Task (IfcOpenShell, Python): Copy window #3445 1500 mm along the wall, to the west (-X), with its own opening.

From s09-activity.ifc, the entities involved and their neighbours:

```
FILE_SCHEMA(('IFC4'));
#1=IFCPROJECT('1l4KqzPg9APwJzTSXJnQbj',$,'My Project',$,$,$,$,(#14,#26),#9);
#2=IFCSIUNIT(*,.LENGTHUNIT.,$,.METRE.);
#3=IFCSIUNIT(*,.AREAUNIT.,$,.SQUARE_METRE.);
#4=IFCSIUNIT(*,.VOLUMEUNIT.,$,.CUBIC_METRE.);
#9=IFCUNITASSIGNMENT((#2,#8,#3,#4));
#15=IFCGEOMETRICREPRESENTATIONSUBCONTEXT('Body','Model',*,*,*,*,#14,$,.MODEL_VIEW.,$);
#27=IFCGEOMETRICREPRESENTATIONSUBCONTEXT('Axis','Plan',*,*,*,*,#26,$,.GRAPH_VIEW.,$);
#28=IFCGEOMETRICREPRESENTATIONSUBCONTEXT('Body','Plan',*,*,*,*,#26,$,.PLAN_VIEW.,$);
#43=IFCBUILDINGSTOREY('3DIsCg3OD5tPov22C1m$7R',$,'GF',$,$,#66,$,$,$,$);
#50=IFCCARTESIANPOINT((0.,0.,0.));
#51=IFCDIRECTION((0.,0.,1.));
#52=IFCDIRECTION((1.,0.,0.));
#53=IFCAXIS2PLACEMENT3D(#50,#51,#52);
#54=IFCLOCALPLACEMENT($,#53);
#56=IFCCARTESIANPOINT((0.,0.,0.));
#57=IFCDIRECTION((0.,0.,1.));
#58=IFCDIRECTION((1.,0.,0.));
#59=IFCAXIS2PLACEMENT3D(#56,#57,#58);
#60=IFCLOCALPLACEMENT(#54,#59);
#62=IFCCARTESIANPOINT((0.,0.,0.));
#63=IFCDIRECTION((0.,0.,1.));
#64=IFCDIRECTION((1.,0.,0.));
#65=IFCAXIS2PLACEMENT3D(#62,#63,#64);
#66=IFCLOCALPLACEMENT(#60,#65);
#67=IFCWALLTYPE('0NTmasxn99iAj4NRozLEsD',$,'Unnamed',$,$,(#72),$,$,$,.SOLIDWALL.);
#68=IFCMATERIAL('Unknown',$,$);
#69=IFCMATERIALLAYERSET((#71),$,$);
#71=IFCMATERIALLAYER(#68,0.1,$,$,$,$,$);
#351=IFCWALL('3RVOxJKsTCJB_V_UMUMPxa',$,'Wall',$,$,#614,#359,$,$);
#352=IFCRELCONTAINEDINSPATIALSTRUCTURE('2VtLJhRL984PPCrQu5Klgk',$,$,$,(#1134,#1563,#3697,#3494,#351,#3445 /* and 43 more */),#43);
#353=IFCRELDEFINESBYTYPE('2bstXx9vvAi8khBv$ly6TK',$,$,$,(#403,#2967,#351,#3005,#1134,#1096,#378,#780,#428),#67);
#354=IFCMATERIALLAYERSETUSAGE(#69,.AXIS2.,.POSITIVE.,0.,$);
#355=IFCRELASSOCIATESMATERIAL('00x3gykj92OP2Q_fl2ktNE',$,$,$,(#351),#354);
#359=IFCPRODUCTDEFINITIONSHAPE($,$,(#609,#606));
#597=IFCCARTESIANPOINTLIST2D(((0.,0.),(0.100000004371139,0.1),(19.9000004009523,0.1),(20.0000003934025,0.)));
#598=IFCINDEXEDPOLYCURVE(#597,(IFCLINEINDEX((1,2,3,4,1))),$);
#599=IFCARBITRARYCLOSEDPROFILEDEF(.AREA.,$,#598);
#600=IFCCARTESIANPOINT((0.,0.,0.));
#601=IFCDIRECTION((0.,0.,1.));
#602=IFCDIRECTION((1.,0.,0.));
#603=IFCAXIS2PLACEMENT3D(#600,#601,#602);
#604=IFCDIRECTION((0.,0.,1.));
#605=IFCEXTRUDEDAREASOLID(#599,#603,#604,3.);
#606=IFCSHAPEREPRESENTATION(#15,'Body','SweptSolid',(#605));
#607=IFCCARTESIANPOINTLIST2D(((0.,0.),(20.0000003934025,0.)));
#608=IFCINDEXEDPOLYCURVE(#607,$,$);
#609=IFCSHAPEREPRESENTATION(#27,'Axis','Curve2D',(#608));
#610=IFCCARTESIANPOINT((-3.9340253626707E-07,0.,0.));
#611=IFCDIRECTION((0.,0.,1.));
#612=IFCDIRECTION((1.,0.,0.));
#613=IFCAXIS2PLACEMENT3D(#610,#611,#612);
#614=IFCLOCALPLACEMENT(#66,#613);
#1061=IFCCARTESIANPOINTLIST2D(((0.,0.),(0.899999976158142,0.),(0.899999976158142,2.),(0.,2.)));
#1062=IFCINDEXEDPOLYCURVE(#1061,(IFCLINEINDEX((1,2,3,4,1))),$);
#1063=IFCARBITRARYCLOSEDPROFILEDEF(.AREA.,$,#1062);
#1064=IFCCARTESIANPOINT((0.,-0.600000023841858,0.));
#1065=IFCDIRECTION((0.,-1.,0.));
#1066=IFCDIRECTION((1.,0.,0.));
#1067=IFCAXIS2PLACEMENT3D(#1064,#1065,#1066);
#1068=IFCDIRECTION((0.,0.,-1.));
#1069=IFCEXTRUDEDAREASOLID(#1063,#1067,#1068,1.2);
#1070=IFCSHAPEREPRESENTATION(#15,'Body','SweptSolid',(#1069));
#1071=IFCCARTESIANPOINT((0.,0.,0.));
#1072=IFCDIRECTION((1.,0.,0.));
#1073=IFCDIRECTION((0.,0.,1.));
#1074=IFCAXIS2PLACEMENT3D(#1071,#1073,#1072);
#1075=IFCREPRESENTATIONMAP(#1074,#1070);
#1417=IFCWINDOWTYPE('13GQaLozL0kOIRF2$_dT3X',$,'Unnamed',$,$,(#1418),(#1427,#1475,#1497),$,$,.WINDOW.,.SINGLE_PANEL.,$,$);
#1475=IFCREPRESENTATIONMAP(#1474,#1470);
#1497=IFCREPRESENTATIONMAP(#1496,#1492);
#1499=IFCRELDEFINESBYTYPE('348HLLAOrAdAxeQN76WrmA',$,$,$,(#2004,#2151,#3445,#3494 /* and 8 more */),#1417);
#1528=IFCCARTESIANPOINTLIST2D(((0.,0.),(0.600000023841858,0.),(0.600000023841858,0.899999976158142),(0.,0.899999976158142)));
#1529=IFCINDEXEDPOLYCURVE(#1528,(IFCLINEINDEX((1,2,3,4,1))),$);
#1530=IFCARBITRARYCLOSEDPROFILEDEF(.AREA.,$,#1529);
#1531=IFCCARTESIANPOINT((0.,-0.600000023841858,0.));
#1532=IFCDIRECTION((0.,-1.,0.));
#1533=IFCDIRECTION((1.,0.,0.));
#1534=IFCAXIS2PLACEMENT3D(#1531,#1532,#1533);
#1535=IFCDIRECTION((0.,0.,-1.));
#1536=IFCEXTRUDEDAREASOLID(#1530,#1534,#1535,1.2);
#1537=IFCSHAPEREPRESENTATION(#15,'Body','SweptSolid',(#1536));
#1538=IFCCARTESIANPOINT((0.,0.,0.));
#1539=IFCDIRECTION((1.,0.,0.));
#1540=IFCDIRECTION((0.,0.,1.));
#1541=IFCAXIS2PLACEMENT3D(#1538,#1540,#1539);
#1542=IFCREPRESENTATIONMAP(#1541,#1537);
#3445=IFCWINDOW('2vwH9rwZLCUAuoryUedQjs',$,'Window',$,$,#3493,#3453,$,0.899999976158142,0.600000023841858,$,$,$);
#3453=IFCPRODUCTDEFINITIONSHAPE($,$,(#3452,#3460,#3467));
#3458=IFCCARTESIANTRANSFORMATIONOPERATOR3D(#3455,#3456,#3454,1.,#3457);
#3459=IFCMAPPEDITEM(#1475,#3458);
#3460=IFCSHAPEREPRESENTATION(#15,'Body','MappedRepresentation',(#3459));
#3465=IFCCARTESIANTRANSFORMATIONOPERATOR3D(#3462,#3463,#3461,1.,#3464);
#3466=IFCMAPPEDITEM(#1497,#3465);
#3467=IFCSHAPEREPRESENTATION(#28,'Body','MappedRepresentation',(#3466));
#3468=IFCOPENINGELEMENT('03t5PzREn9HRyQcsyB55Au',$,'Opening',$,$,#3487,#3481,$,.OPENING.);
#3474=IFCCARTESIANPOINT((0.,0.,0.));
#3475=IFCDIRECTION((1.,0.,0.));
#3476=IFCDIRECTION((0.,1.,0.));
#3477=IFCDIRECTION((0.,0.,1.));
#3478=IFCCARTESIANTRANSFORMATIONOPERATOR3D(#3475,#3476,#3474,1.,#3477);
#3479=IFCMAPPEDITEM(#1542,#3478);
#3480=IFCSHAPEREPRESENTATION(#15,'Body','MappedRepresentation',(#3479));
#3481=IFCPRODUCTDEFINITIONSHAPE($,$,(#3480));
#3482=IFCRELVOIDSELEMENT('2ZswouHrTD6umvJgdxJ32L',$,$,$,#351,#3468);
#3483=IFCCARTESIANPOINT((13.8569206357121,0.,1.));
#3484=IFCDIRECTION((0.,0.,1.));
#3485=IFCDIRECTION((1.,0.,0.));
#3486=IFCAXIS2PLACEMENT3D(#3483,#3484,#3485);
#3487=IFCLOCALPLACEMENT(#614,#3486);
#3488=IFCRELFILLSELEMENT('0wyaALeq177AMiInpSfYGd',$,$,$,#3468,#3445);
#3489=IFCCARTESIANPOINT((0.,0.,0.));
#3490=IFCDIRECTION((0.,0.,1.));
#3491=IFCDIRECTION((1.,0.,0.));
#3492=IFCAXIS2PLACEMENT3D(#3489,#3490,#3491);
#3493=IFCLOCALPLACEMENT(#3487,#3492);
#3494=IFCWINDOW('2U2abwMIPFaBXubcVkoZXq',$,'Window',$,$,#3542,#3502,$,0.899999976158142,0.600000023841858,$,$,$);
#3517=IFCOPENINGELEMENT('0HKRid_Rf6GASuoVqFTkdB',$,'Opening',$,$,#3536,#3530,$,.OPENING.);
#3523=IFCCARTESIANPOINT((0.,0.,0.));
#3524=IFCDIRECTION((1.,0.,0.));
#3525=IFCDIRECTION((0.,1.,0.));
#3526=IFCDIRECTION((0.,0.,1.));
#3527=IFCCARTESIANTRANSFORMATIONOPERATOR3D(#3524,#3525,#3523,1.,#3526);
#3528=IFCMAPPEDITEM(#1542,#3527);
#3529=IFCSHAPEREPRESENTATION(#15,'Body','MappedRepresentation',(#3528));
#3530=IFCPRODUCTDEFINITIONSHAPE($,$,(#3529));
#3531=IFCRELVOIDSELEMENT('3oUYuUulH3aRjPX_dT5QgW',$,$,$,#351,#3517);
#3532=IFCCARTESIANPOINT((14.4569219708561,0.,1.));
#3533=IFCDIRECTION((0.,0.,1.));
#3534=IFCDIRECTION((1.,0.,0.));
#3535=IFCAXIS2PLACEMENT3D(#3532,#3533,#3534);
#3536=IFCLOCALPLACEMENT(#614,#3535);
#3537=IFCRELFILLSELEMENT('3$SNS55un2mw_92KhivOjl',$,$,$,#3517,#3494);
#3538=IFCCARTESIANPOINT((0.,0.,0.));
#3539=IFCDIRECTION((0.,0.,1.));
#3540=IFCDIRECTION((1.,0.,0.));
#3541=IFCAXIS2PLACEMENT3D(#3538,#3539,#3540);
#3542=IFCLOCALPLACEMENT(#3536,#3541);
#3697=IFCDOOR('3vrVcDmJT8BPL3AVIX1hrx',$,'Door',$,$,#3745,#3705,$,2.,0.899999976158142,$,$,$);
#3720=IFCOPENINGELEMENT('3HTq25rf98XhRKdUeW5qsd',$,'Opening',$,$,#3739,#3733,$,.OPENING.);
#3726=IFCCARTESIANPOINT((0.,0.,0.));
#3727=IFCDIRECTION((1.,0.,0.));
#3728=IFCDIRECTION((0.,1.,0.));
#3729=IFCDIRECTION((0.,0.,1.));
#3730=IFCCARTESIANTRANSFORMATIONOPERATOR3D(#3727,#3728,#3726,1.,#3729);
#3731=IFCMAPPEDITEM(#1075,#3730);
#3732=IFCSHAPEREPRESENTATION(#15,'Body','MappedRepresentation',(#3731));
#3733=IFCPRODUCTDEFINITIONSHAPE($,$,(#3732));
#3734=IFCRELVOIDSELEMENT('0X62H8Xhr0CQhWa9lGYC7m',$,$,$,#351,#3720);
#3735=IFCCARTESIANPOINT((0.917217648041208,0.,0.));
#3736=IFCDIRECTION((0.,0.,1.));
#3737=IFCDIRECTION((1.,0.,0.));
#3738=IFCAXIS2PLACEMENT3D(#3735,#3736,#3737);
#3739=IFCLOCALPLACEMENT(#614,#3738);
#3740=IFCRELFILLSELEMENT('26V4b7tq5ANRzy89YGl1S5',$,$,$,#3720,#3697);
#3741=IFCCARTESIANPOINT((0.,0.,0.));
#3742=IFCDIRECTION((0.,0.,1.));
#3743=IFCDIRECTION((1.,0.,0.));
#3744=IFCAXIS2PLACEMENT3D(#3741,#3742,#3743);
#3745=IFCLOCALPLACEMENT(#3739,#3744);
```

```python
import ifcopenshell
import ifcopenshell.api.feature
import ifcopenshell.api.geometry
import ifcopenshell.api.root
import ifcopenshell.geom
import ifcopenshell.util.element
import ifcopenshell.util.placement
import ifcopenshell.util.shape
import ifcopenshell.util.unit

model = ifcopenshell.open("s09-activity.ifc")
unit_scale = ifcopenshell.util.unit.calculate_unit_scale(model)
settings = ifcopenshell.geom.settings()


def volume(element):
    """Net volume in cubic metres, openings subtracted."""
    shape = ifcopenshell.geom.create_shape(settings, element)
    return ifcopenshell.util.shape.get_volume(shape.geometry)


window = model.by_id(3445)
opening = window.FillsVoids[0].RelatingOpeningElement
wall = opening.VoidsElements[0].RelatingBuildingElement
before = volume(wall)
shift = ifcopenshell.util.placement.get_local_placement(wall.ObjectPlacement)[:3, 0] * -1.5 / unit_scale

# copy_class copies the void relationship, type, container and properties, but no geometry.
new_opening = ifcopenshell.api.root.copy_class(model, product=opening)
new_opening.Representation = ifcopenshell.util.element.copy_deep(
    model, opening.Representation, exclude=["IfcGeometricRepresentationContext", "IfcRepresentationMap"]
)
new_window = ifcopenshell.api.root.copy_class(model, product=window)
new_window.Representation = ifcopenshell.util.element.copy_deep(
    model, window.Representation, exclude=["IfcGeometricRepresentationContext", "IfcRepresentationMap"]
)
ifcopenshell.api.feature.add_filling(model, opening=new_opening, element=new_window)

for old, new in ((opening, new_opening), (window, new_window)):
    matrix = ifcopenshell.util.placement.get_local_placement(old.ObjectPlacement)
    matrix[:3, 3] += shift
    ifcopenshell.api.geometry.edit_object_placement(model, product=new, matrix=matrix, is_si=False)

after = volume(wall)

print(f"wall volume {before:.3f} -> {after:.3f} m3")

model.write("s09-activity_edited.ifc")
```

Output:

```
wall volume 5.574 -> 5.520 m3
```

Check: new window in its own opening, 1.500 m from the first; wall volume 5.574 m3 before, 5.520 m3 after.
